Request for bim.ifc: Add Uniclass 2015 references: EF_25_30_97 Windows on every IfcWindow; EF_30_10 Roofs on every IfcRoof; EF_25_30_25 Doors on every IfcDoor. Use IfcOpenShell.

First a look at what the model holds.

```python
import ifcopenshell

model = ifcopenshell.open("bim.ifc")
print(model.schema)
print("classifications:", [c.Name for c in model.by_type("IfcClassification")])
for ifc_class in ("IfcDoor", "IfcRoof", "IfcStair", "IfcWall", "IfcWindow"):
    print(ifc_class, len(model.by_type(ifc_class)))
```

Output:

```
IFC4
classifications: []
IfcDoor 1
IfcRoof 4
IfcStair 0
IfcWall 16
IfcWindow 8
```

```python
import ifcopenshell
import ifcopenshell.api.classification

model = ifcopenshell.open("bim.ifc")

system = ifcopenshell.api.classification.add_classification(model, classification="Uniclass 2015")

codes = {
    "IfcWindow": ("EF_25_30_97", "Windows"),
    "IfcRoof": ("EF_30_10", "Roofs"),
    "IfcDoor": ("EF_25_30_25", "Doors"),
}
for ifc_class, (code, name) in codes.items():
    products = model.by_type(ifc_class)
    ifcopenshell.api.classification.add_reference(
        model, products=products, classification=system, identification=code, name=name
    )
    print(code, len(products))

model.write("bim-out.ifc")
```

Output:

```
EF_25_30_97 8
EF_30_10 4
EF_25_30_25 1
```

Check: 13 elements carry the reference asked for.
